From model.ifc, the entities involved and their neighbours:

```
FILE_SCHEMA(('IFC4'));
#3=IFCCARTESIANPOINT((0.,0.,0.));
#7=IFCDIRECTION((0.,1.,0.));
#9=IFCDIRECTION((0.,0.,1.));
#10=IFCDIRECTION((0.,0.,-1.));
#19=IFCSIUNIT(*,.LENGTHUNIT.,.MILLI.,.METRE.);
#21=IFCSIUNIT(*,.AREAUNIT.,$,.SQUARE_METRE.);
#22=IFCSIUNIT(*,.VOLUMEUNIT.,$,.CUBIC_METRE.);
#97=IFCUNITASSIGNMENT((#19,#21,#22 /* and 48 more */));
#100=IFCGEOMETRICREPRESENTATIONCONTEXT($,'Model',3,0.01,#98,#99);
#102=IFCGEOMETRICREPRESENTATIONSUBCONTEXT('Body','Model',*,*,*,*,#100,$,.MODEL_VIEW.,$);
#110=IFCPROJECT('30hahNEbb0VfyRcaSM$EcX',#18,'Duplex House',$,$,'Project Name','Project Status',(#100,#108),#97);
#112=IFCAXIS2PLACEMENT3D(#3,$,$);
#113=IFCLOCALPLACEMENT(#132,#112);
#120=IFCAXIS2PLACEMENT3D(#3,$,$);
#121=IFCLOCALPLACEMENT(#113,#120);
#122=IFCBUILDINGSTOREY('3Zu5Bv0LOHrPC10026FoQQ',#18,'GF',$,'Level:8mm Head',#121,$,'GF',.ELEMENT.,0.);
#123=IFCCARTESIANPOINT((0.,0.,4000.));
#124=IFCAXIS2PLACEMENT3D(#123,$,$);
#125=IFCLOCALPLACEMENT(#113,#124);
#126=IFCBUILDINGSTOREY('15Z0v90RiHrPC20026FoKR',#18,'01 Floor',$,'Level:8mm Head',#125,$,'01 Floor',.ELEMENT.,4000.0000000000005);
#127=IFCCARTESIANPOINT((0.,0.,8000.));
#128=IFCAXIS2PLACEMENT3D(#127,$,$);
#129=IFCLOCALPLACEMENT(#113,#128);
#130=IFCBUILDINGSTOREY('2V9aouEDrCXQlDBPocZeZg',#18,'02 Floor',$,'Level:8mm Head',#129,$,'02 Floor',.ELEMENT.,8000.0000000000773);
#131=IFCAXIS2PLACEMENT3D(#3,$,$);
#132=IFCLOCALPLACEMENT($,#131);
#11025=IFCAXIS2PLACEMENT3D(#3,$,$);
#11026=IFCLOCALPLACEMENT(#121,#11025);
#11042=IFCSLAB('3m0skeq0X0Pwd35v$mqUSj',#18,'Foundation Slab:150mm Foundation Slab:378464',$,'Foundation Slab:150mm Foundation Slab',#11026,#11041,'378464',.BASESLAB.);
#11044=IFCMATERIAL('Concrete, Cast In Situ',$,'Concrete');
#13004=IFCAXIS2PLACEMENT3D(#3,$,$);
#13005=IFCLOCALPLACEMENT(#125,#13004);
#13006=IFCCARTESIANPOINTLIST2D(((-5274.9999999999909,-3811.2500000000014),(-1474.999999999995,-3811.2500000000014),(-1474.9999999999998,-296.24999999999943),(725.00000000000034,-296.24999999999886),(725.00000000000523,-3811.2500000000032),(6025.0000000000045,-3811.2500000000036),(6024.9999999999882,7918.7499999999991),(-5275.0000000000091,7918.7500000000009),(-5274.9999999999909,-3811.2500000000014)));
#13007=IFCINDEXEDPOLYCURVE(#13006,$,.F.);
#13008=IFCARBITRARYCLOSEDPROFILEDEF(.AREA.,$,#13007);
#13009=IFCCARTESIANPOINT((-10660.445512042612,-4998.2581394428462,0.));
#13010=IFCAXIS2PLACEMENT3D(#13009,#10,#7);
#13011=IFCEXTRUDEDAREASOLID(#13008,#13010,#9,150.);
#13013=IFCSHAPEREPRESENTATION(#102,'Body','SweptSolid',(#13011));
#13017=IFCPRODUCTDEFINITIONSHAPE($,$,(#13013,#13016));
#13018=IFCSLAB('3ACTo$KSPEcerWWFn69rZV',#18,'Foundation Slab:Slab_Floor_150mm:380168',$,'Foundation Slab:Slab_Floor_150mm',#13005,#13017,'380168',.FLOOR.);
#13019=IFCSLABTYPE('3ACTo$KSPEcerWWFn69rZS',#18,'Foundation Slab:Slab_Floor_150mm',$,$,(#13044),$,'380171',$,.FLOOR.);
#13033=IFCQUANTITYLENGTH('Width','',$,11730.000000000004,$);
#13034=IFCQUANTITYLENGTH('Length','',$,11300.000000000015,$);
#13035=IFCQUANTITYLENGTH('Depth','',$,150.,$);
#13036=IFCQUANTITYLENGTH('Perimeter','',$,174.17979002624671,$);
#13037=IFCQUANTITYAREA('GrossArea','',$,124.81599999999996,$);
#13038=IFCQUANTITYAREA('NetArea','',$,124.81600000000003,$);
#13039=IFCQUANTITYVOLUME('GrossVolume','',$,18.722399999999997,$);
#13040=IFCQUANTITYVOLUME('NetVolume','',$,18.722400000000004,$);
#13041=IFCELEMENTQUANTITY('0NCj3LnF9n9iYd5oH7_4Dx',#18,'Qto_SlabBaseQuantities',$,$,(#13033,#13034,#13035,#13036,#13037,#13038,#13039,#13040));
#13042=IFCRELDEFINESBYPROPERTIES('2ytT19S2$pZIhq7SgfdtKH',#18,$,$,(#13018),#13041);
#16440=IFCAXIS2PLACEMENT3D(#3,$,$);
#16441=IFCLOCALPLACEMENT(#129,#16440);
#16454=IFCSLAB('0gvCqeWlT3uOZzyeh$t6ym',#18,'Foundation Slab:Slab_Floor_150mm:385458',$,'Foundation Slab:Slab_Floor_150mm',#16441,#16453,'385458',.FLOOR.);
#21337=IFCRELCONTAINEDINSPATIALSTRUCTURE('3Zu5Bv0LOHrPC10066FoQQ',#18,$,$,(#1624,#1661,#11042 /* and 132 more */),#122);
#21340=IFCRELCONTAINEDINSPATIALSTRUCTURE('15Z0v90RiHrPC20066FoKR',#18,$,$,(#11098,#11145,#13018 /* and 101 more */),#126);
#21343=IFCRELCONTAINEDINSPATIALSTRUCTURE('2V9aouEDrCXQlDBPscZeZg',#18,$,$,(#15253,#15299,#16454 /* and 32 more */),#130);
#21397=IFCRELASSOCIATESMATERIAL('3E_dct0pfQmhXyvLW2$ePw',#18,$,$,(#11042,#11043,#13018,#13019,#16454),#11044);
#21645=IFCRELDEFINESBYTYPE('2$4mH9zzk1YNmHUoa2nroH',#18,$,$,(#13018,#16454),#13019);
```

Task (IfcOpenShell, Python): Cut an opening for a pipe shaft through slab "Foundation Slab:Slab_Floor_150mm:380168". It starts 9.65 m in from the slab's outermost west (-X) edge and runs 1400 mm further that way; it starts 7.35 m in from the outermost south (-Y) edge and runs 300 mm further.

```python
import numpy as np
import ifcopenshell
import ifcopenshell.api.feature
import ifcopenshell.api.geometry
import ifcopenshell.api.pset
import ifcopenshell.api.root
import ifcopenshell.geom
import ifcopenshell.util.element
import ifcopenshell.util.placement
import ifcopenshell.util.representation
import ifcopenshell.util.shape
import ifcopenshell.util.unit

model = ifcopenshell.open("model.ifc")
unit_scale = ifcopenshell.util.unit.calculate_unit_scale(model)
area_scale = ifcopenshell.util.unit.calculate_unit_scale(model, "AREAUNIT")
volume_scale = ifcopenshell.util.unit.calculate_unit_scale(model, "VOLUMEUNIT")
settings = ifcopenshell.geom.settings()


def volume(element):
    """Net volume in cubic metres, openings subtracted."""
    shape = ifcopenshell.geom.create_shape(settings, element)
    return ifcopenshell.util.shape.get_volume(shape.geometry)


slab = model.by_guid("3ACTo$KSPEcerWWFn69rZV")
before = volume(slab)

# Extent in the slab's own axes, in metres. The edges named are its -X and -Y sides.
slab_shape = ifcopenshell.geom.create_shape(settings, slab)
vertices = ifcopenshell.util.shape.get_vertices(slab_shape.geometry)
x_min, y_min, bottom = vertices.min(axis=0)
top = vertices[:, 2].max()

opening = ifcopenshell.api.root.create_entity(model, ifc_class="IfcOpeningElement", name="Pipe shaft opening", predefined_type="OPENING")
context = ifcopenshell.util.representation.get_context(model, "Model", "Body", "MODEL_VIEW")
width, depth = 1.4, 0.3
outline = [(0.0, 0.0), (width, 0.0), (width, depth), (0.0, depth), (0.0, 0.0)]
# Overshoot both faces by 50 mm so the cut is clean.
shape = ifcopenshell.api.geometry.add_slab_representation(
    model, context=context, depth=top - bottom + 0.1, polyline=outline
)
ifcopenshell.api.geometry.assign_representation(model, product=opening, representation=shape)

matrix = ifcopenshell.util.placement.get_local_placement(slab.ObjectPlacement)
matrix[:, 3] = matrix @ np.append(np.array([x_min + 9.65, y_min + 7.35, bottom - 0.05]) / unit_scale, 1.0)
ifcopenshell.api.geometry.edit_object_placement(model, product=opening, matrix=matrix, is_si=False)
ifcopenshell.api.feature.add_feature(model, feature=opening, element=slab)

after = volume(slab)

# Update the slab's stored quantities.
qto = model.by_id(ifcopenshell.util.element.get_pset(slab, "Qto_SlabBaseQuantities", should_inherit=False)["id"])
ifcopenshell.api.pset.edit_qto(model, qto=qto, properties={
    "NetArea": after / (top - bottom) / area_scale,
    "NetVolume": after / volume_scale,
})

print(f"slab volume {before:.3f} -> {after:.3f} m3")

model.write("model_rev.ifc")
```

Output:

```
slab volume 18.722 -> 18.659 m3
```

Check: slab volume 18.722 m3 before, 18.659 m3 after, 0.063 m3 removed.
